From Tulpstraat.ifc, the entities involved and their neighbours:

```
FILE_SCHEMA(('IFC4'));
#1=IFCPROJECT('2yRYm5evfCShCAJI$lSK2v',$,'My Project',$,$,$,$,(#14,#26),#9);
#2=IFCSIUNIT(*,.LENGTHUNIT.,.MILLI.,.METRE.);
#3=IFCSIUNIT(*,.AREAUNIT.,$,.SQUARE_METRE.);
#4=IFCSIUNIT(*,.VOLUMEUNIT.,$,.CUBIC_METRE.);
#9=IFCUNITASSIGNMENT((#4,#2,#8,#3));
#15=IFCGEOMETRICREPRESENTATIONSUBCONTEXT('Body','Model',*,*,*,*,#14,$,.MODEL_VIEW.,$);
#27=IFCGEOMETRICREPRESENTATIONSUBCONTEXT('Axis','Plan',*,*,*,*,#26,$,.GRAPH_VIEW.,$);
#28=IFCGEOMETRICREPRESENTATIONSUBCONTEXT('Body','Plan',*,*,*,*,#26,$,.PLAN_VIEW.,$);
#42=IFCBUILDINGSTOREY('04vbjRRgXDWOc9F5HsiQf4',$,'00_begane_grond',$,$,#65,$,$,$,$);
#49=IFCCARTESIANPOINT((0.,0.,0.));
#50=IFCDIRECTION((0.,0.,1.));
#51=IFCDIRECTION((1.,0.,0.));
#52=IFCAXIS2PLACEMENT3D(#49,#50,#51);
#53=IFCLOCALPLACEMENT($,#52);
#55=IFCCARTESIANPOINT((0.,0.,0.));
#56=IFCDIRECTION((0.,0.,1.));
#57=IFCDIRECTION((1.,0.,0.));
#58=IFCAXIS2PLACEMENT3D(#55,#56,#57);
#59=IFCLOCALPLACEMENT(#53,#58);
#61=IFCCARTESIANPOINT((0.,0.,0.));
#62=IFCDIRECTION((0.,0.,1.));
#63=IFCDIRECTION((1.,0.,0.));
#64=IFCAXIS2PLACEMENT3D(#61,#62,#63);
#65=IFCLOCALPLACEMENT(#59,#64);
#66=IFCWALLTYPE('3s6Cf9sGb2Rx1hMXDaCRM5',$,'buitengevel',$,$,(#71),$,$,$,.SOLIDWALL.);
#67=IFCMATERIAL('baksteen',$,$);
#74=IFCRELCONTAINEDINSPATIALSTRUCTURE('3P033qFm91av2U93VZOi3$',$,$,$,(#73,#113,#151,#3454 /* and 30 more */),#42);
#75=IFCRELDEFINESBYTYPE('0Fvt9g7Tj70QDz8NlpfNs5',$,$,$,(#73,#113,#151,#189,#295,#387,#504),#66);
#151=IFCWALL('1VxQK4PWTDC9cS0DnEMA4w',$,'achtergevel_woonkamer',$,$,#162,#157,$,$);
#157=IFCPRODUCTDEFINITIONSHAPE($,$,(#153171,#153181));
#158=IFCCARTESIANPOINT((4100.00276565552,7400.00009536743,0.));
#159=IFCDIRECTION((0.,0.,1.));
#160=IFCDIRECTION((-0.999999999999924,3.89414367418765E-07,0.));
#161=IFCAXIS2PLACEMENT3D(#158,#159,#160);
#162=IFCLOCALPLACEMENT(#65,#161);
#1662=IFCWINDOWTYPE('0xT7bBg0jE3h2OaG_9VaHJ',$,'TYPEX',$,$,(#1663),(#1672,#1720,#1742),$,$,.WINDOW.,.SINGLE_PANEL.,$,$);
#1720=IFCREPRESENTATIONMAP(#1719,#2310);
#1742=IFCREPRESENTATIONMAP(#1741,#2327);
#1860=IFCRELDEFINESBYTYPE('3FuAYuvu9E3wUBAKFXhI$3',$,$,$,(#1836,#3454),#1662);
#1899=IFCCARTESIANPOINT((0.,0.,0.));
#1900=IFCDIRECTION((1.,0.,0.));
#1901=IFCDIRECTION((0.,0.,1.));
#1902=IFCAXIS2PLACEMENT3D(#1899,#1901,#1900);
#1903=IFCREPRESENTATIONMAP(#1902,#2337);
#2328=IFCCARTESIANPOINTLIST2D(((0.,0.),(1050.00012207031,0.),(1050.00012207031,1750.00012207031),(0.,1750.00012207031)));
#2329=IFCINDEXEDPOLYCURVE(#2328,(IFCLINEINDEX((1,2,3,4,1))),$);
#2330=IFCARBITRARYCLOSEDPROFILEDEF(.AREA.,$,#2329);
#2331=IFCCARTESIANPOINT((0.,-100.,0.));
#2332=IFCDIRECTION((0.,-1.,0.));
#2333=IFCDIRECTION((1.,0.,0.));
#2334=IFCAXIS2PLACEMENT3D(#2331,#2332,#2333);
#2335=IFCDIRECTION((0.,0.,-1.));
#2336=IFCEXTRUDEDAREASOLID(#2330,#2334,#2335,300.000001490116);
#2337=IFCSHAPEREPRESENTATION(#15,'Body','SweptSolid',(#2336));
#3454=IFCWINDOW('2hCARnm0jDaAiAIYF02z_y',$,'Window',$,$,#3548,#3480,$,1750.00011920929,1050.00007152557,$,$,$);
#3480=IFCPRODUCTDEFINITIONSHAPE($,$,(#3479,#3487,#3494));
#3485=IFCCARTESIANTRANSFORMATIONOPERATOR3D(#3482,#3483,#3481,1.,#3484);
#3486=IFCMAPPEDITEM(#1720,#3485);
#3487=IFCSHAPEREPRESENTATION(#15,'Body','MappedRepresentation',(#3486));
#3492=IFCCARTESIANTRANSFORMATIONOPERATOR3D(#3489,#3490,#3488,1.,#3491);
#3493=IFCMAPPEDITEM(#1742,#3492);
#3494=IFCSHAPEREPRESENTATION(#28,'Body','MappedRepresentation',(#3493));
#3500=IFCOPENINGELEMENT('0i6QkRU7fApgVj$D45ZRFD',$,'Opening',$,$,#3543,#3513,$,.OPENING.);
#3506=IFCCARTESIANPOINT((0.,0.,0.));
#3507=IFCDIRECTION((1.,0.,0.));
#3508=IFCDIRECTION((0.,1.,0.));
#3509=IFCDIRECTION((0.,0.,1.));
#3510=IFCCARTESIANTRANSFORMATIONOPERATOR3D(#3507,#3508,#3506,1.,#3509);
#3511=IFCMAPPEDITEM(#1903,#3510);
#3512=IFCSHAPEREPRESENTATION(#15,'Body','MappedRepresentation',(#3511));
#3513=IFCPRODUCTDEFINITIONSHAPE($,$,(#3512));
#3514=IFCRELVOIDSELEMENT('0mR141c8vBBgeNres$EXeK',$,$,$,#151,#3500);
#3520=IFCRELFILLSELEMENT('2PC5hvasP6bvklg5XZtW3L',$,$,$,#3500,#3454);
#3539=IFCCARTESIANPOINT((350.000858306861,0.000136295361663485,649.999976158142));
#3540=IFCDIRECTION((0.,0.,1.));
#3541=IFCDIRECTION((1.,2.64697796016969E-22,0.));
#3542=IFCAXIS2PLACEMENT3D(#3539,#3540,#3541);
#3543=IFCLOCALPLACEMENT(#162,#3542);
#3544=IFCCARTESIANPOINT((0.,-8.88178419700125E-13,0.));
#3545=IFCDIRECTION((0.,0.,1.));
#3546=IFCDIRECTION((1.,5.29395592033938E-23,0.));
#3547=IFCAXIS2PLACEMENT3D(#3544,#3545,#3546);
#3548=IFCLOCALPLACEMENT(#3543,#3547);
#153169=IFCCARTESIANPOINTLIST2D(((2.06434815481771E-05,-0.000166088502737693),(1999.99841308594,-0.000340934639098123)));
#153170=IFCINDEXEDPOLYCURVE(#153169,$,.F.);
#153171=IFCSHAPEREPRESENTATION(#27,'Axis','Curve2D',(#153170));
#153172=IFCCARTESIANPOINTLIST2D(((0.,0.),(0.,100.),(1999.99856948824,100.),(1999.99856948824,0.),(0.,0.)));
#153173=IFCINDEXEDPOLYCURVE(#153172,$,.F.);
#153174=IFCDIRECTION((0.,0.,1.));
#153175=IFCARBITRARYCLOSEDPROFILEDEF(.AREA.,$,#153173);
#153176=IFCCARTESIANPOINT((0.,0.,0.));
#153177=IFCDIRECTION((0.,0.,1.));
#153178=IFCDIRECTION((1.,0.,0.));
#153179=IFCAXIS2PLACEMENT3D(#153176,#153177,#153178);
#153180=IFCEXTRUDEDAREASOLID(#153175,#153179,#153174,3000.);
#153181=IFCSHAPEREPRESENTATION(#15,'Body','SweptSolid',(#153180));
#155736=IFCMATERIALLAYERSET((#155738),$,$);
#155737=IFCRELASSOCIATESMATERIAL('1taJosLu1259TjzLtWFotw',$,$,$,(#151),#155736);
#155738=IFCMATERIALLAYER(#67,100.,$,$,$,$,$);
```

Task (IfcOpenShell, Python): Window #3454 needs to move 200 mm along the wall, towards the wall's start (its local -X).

```python
import ifcopenshell
import ifcopenshell.api.geometry
import ifcopenshell.util.placement
import ifcopenshell.util.unit

model = ifcopenshell.open("Tulpstraat.ifc")
unit_scale = ifcopenshell.util.unit.calculate_unit_scale(model)

window = model.by_guid("2hCARnm0jDaAiAIYF02z_y")
opening = window.FillsVoids[0].RelatingOpeningElement
wall = opening.VoidsElements[0].RelatingBuildingElement

wall_matrix = ifcopenshell.util.placement.get_local_placement(wall.ObjectPlacement)
shift = wall_matrix[:3, 0] * -0.2 / unit_scale
before = ifcopenshell.util.placement.get_local_placement(window.ObjectPlacement)[:3, 3].copy()

# The window is placed relative to its opening, so it follows when the opening moves.
matrix = ifcopenshell.util.placement.get_local_placement(opening.ObjectPlacement)
matrix[:3, 3] += shift
ifcopenshell.api.geometry.edit_object_placement(
    model, product=opening, matrix=matrix, is_si=False, should_transform_children=True
)

after = ifcopenshell.util.placement.get_local_placement(window.ObjectPlacement)[:3, 3]
print("window moved by", (after - before).round(3) + 0.0)

model.write("Tulpstraat_edited.ifc")
```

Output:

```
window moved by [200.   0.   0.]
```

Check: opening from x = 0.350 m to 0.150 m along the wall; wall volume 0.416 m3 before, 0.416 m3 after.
